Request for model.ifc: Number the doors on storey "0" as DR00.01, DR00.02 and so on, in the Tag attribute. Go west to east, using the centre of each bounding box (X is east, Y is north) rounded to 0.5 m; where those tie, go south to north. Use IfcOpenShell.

First a look at what the model holds.

```python
import ifcopenshell
import ifcopenshell.util.element
import ifcopenshell.util.placement

model = ifcopenshell.open("model.ifc")
print(model.schema)
storey = next(s for s in model.by_type("IfcBuildingStorey") if s.Name == "0")
doors = [e for e in ifcopenshell.util.element.get_decomposition(storey) if e.is_a("IfcDoor")]
for e in sorted(doors, key=lambda e: e.id()):
    origin = ifcopenshell.util.placement.get_local_placement(e.ObjectPlacement)[:3, 3]
    print(e.id(), e.Tag, e.Name, origin.round(2) + 0.0, sep=" | ")
```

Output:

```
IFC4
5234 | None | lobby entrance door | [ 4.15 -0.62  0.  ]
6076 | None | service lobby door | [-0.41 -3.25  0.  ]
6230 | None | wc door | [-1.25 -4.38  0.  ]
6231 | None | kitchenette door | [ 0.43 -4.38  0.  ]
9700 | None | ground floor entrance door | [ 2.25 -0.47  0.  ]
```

```python
import ifcopenshell
import ifcopenshell.geom
import ifcopenshell.util.element
import ifcopenshell.util.shape

model = ifcopenshell.open("model.ifc")
settings = ifcopenshell.geom.settings()
settings.set("use-world-coords", True)


def centre(element):
    shape = ifcopenshell.geom.create_shape(settings, element)
    return ifcopenshell.util.shape.get_bbox_centroid(shape.geometry)


storey = next(s for s in model.by_type("IfcBuildingStorey") if s.Name == "0")
doors = [e for e in ifcopenshell.util.element.get_decomposition(storey) if e.is_a("IfcDoor")]

# Insertion points can sit at a corner or the storey origin, so sort by the geometry (in metres).
centres = {e: centre(e) for e in doors}
doors.sort(key=lambda e: (round(centres[e][0] / 0.5), centres[e][1]))

for i, e in enumerate(doors, start=1):
    number = f"DR00.{i:02d}"
    e.Tag = number
    print(e.id(), number)

model.write("model-out.ifc")
```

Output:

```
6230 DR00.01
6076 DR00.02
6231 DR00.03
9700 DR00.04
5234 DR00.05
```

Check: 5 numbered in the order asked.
